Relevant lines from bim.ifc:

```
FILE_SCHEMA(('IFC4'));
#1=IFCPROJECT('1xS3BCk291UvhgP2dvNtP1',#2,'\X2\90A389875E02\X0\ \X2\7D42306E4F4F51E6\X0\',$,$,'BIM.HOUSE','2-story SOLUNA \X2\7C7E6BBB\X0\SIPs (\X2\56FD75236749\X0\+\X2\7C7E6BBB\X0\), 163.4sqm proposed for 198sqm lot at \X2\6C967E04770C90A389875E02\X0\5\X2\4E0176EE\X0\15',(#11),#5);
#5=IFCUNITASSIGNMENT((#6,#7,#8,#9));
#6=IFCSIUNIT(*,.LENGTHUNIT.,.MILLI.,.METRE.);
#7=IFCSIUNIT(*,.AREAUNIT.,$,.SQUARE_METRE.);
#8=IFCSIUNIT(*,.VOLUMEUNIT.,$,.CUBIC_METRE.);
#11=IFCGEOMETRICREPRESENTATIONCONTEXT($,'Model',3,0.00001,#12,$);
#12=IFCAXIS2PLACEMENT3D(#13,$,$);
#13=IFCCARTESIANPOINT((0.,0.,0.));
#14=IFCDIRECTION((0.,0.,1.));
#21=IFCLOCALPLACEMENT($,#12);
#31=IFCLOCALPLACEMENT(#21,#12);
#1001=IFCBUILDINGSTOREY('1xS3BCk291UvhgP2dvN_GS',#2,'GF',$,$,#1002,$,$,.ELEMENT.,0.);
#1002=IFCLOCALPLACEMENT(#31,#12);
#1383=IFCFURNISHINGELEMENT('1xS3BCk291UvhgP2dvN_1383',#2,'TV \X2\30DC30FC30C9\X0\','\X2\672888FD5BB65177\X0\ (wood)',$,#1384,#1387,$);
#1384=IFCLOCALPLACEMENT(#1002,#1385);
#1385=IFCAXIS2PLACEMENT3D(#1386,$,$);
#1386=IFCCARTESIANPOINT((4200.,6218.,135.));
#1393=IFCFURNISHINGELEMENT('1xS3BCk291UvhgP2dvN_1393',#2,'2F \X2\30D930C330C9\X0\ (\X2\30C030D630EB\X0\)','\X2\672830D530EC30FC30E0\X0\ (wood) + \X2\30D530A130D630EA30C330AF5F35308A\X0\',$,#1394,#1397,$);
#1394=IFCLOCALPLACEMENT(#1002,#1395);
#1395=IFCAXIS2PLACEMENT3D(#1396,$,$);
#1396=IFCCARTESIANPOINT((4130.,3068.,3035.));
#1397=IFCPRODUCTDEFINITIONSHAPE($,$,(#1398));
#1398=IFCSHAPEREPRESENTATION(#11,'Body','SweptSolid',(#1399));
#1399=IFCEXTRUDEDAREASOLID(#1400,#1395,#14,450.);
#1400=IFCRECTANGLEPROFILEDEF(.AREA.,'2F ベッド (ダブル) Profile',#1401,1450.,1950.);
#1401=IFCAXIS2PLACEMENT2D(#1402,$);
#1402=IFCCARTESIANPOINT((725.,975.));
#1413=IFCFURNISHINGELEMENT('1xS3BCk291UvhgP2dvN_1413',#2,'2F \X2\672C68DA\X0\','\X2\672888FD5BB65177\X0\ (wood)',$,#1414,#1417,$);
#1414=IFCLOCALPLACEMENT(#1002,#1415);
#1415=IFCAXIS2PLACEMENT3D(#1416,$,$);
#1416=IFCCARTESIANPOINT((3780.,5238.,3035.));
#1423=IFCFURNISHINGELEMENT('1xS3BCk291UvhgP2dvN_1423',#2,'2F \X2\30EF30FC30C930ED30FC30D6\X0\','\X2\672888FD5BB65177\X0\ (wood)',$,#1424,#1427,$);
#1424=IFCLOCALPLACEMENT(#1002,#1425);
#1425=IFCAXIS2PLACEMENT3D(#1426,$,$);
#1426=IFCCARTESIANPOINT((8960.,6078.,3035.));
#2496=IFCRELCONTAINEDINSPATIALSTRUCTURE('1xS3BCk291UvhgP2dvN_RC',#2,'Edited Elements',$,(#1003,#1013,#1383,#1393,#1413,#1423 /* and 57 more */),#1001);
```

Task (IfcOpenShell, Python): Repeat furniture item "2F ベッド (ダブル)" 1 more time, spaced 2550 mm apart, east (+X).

```python
import numpy as np
import ifcopenshell
import ifcopenshell.api.geometry
import ifcopenshell.api.root
import ifcopenshell.util.element
import ifcopenshell.util.placement
import ifcopenshell.util.unit

model = ifcopenshell.open("bim.ifc")
unit_scale = ifcopenshell.util.unit.calculate_unit_scale(model)


def reuse_history(source, copy):
    """copy_class also copies each property set's owner history, people and application; keep the originals."""
    for rel in copy.IsDefinedBy:
        if rel.is_a("IfcRelDefinesByProperties") and (history := rel.RelatingPropertyDefinition.OwnerHistory):
            rel.RelatingPropertyDefinition.OwnerHistory = source.OwnerHistory
            ifcopenshell.util.element.remove_deep2(model, history)


source = model.by_guid("1xS3BCk291UvhgP2dvN_1393")
base = ifcopenshell.util.placement.get_local_placement(source.ObjectPlacement)
step = np.array([1.0, 0.0, 0.0]) * 2.55 / unit_scale

for i in range(1, 2):
    copy = ifcopenshell.api.root.copy_class(model, product=source)
    copy.Representation = ifcopenshell.util.element.copy_deep(
        model, source.Representation, exclude=["IfcGeometricRepresentationContext", "IfcRepresentationMap"]
    )
    reuse_history(source, copy)
    matrix = base.copy()
    matrix[:3, 3] += i * step
    print("added at", matrix[:3, 3].round(3) + 0.0)
    ifcopenshell.api.geometry.edit_object_placement(model, product=copy, matrix=matrix, is_si=False)

model.write("bim_rev.ifc")
```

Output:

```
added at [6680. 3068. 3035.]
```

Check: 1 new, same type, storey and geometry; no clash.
